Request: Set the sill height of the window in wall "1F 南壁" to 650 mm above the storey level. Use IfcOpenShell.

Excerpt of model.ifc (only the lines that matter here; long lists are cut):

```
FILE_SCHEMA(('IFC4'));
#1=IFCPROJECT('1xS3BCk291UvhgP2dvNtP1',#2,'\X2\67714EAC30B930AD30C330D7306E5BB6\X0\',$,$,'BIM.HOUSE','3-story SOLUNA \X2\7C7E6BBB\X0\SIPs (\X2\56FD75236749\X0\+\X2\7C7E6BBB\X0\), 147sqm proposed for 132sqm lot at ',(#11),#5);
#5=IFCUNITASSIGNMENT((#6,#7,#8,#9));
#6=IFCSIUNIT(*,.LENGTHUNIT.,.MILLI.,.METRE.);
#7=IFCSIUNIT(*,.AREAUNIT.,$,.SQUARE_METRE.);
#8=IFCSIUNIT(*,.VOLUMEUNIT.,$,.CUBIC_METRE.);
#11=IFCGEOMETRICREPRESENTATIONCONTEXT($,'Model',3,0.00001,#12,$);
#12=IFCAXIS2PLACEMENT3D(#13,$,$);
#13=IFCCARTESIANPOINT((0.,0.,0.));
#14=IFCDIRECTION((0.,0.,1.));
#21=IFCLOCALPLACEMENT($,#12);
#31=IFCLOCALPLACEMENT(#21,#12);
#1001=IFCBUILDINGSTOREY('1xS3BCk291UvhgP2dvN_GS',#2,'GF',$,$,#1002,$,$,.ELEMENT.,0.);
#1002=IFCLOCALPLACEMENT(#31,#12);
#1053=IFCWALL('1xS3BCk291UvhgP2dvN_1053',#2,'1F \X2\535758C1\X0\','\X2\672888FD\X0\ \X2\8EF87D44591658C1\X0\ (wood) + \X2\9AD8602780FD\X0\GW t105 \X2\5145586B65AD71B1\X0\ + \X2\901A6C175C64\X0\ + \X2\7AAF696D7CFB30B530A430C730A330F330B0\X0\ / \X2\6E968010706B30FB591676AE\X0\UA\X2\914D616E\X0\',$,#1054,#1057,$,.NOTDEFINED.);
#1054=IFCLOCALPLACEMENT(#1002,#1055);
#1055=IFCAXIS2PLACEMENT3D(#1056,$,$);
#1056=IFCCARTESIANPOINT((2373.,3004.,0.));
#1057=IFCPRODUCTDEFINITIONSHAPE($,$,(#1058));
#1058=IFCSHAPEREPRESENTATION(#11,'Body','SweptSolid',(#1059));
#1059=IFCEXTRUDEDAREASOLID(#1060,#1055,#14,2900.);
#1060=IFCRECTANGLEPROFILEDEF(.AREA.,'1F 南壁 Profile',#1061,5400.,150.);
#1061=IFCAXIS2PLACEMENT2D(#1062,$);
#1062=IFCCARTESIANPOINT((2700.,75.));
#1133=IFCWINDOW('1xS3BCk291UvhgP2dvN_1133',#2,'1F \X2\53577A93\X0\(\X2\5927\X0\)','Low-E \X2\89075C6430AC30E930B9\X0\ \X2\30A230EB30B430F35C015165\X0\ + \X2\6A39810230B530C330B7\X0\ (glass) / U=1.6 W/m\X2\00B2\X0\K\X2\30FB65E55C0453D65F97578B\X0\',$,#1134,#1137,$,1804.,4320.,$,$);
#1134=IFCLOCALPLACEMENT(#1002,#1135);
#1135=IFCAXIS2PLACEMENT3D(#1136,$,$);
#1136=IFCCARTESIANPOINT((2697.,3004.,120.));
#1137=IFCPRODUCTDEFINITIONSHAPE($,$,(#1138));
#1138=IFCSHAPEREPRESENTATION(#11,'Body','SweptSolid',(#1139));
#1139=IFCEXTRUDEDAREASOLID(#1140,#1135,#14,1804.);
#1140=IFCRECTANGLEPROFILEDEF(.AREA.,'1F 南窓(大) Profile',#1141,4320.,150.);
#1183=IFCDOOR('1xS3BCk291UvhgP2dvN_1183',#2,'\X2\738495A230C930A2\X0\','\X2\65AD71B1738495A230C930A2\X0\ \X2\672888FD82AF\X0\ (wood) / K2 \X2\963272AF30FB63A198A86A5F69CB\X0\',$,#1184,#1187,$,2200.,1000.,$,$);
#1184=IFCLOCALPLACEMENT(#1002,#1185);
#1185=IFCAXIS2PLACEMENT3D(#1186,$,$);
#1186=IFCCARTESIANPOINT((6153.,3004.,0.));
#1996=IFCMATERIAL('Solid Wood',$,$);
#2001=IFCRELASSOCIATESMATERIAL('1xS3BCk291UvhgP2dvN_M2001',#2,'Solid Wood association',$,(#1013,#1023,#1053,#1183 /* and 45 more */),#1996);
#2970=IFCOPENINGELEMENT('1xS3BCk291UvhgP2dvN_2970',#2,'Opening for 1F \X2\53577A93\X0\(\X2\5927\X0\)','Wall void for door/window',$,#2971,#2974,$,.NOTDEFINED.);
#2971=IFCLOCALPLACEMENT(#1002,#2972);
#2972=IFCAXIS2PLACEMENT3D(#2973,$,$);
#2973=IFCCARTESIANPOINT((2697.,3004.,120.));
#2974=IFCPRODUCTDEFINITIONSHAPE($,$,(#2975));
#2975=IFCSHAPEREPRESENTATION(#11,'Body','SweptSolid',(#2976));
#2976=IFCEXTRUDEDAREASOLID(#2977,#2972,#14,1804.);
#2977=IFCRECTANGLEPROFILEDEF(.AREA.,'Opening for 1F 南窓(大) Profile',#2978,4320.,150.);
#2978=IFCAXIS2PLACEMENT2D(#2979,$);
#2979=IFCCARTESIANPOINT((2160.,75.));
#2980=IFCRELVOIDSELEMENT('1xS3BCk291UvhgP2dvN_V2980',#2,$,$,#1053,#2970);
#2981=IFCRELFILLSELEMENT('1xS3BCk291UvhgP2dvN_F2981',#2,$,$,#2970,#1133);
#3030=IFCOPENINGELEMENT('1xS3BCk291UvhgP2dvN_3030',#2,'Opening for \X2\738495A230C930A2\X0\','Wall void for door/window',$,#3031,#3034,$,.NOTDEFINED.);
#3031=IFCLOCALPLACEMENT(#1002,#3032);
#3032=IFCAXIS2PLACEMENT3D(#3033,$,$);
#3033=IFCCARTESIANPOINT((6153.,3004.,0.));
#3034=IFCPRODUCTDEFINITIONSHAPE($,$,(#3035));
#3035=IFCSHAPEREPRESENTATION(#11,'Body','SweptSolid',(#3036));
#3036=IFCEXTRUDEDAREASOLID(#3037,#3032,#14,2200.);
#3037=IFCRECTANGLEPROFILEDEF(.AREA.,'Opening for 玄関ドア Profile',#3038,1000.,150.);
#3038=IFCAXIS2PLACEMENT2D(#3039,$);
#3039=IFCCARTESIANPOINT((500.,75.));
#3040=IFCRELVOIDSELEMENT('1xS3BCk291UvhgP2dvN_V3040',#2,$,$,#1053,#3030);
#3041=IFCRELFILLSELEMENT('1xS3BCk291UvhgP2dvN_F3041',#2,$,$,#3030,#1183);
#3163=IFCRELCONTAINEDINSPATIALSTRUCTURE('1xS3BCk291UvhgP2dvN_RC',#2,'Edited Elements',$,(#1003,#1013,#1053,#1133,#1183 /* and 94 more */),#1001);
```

```python
import numpy as np
import ifcopenshell
import ifcopenshell.api.geometry
import ifcopenshell.geom
import ifcopenshell.util.element
import ifcopenshell.util.placement
import ifcopenshell.util.shape
import ifcopenshell.util.unit

model = ifcopenshell.open("model.ifc")
unit_scale = ifcopenshell.util.unit.calculate_unit_scale(model)

window = model.by_id(1133)
opening = window.FillsVoids[0].RelatingOpeningElement
storey = ifcopenshell.util.element.get_container(window, ifc_class="IfcBuildingStorey")
level = ifcopenshell.util.placement.get_local_placement(storey.ObjectPlacement)[2, 3]

# The opening's origin need not be at the sill, so measure its lowest point.
shape = ifcopenshell.geom.create_shape(ifcopenshell.geom.settings(), opening)
bottom = ifcopenshell.util.shape.get_shape_bottom_elevation(shape, shape.geometry) / unit_scale
dz = level + 0.65 / unit_scale - bottom

shift = np.array([0.0, 0.0, dz])
# The window is not placed relative to its opening, so move both.
for product in (opening, window):
    matrix = ifcopenshell.util.placement.get_local_placement(product.ObjectPlacement)
    matrix[:3, 3] += shift
    ifcopenshell.api.geometry.edit_object_placement(model, product=product, matrix=matrix, is_si=False)

print(f"moved by {dz * unit_scale:+.3f} m")

model.write("model_edited.ifc")
```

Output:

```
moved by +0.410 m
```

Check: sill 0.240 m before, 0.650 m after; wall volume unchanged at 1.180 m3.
